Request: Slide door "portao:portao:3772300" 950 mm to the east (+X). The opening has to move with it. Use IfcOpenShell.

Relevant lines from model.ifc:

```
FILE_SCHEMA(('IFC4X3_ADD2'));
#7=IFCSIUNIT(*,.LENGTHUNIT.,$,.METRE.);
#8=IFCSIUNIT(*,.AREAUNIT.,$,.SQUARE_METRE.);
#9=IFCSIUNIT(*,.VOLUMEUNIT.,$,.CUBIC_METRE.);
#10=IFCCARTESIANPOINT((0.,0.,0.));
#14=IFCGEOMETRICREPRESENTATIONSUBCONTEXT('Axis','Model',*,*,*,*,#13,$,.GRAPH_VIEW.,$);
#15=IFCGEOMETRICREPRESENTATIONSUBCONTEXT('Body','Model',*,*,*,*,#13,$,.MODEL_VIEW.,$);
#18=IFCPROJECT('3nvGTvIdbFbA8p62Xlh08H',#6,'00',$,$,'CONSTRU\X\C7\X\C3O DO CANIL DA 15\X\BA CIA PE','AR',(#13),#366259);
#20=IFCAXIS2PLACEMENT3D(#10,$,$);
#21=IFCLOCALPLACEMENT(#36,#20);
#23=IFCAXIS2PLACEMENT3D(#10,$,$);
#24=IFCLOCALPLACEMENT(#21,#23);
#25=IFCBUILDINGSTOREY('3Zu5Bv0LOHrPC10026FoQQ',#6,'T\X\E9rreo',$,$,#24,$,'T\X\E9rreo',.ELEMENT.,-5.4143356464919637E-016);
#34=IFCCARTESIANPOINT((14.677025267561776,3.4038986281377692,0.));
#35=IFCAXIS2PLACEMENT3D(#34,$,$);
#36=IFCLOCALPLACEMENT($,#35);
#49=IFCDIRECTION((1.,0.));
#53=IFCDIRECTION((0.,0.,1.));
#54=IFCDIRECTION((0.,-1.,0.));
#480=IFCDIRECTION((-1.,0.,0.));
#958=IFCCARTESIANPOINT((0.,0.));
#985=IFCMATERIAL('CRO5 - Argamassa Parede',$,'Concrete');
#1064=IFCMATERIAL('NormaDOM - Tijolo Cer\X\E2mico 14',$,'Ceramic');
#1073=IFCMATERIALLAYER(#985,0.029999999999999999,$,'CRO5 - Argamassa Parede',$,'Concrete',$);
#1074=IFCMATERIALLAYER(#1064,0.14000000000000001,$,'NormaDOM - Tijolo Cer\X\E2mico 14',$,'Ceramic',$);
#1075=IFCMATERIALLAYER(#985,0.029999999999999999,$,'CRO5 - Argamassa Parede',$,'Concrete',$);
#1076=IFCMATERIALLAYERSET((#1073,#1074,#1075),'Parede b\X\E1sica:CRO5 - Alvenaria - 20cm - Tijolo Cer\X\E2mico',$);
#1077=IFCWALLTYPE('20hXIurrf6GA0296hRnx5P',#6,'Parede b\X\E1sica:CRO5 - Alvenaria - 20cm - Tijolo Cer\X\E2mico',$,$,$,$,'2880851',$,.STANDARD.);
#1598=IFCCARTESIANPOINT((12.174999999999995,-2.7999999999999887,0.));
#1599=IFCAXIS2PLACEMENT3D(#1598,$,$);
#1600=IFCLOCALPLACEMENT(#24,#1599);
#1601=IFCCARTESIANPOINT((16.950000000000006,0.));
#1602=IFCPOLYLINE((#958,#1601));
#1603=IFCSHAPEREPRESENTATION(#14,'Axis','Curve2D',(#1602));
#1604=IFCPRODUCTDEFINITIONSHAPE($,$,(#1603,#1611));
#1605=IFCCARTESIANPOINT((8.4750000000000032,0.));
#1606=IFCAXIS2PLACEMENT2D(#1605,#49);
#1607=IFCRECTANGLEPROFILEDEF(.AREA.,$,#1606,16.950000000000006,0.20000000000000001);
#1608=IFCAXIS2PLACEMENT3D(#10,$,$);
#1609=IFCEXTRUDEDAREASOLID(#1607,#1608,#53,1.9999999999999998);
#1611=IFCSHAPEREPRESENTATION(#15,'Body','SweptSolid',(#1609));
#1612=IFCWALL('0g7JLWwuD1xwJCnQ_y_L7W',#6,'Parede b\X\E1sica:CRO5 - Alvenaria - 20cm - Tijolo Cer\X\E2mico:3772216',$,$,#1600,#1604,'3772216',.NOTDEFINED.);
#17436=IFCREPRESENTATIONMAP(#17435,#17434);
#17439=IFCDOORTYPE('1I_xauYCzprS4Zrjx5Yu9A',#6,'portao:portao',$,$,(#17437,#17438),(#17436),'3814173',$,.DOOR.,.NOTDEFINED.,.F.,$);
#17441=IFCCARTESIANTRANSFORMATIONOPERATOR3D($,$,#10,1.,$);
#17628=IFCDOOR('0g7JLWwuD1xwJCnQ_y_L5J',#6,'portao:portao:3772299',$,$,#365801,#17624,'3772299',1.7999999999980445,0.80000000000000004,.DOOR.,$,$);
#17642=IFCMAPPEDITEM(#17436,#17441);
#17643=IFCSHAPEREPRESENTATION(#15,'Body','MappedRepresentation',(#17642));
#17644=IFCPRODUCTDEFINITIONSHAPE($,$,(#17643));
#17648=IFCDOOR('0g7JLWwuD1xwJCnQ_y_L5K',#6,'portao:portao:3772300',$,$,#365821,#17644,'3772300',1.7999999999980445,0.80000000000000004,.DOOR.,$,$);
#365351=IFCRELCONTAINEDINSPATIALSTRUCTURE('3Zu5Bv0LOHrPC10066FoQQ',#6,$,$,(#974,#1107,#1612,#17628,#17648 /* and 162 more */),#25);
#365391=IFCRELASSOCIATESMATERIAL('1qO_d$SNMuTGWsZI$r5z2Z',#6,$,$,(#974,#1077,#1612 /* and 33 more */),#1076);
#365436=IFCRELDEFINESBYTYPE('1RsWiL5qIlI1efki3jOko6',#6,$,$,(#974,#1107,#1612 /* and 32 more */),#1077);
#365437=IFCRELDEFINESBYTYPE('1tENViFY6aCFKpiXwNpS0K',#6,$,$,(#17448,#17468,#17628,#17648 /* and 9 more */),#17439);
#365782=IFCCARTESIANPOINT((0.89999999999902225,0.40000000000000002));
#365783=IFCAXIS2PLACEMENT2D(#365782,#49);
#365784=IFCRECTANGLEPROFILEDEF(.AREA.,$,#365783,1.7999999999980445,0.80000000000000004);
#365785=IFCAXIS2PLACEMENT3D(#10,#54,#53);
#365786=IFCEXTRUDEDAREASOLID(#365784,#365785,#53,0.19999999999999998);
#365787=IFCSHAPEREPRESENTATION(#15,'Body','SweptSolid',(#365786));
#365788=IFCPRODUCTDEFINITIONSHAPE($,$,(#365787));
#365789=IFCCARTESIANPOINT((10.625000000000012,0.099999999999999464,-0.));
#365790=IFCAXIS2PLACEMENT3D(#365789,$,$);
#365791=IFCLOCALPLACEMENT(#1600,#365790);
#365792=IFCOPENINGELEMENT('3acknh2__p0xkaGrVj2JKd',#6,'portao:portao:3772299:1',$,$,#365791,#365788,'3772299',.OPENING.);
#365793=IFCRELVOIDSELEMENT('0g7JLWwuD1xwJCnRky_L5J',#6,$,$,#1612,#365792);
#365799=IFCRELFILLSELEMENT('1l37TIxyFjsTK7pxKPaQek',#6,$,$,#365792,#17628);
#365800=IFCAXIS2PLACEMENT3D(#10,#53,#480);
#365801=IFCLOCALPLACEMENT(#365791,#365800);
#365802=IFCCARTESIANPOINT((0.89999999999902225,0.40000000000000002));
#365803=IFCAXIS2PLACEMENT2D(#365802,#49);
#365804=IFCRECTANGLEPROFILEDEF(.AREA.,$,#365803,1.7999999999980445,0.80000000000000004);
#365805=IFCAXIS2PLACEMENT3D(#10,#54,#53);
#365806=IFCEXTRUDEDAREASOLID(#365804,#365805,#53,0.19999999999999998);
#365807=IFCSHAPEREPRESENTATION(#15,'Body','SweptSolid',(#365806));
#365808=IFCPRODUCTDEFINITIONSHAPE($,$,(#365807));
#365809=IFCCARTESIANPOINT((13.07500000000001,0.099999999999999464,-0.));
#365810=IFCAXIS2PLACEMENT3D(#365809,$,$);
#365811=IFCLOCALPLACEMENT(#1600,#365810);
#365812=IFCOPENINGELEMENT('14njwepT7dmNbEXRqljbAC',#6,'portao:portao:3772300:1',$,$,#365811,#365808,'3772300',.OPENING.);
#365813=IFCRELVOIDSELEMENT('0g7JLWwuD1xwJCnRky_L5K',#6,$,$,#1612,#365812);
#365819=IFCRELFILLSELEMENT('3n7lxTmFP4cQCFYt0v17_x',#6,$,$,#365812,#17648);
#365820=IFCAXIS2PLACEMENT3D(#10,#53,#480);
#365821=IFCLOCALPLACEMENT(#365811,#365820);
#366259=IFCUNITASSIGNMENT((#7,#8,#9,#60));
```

```python
import ifcopenshell
import ifcopenshell.api.geometry
import ifcopenshell.util.placement
import ifcopenshell.util.unit

model = ifcopenshell.open("model.ifc")
unit_scale = ifcopenshell.util.unit.calculate_unit_scale(model)

door = model.by_guid("0g7JLWwuD1xwJCnQ_y_L5K")
opening = door.FillsVoids[0].RelatingOpeningElement
wall = opening.VoidsElements[0].RelatingBuildingElement

wall_matrix = ifcopenshell.util.placement.get_local_placement(wall.ObjectPlacement)
shift = wall_matrix[:3, 0] * 0.95 / unit_scale
before = ifcopenshell.util.placement.get_local_placement(door.ObjectPlacement)[:3, 3].copy()

# The door is placed relative to its opening, so it follows when the opening moves.
matrix = ifcopenshell.util.placement.get_local_placement(opening.ObjectPlacement)
matrix[:3, 3] += shift
ifcopenshell.api.geometry.edit_object_placement(
    model, product=opening, matrix=matrix, is_si=False, should_transform_children=True
)

after = ifcopenshell.util.placement.get_local_placement(door.ObjectPlacement)[:3, 3]
print("door moved by", (after - before).round(3) + 0.0)

model.write("model_rev.ifc")
```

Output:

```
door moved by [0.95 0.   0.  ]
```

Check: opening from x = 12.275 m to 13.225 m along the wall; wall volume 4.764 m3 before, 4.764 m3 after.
